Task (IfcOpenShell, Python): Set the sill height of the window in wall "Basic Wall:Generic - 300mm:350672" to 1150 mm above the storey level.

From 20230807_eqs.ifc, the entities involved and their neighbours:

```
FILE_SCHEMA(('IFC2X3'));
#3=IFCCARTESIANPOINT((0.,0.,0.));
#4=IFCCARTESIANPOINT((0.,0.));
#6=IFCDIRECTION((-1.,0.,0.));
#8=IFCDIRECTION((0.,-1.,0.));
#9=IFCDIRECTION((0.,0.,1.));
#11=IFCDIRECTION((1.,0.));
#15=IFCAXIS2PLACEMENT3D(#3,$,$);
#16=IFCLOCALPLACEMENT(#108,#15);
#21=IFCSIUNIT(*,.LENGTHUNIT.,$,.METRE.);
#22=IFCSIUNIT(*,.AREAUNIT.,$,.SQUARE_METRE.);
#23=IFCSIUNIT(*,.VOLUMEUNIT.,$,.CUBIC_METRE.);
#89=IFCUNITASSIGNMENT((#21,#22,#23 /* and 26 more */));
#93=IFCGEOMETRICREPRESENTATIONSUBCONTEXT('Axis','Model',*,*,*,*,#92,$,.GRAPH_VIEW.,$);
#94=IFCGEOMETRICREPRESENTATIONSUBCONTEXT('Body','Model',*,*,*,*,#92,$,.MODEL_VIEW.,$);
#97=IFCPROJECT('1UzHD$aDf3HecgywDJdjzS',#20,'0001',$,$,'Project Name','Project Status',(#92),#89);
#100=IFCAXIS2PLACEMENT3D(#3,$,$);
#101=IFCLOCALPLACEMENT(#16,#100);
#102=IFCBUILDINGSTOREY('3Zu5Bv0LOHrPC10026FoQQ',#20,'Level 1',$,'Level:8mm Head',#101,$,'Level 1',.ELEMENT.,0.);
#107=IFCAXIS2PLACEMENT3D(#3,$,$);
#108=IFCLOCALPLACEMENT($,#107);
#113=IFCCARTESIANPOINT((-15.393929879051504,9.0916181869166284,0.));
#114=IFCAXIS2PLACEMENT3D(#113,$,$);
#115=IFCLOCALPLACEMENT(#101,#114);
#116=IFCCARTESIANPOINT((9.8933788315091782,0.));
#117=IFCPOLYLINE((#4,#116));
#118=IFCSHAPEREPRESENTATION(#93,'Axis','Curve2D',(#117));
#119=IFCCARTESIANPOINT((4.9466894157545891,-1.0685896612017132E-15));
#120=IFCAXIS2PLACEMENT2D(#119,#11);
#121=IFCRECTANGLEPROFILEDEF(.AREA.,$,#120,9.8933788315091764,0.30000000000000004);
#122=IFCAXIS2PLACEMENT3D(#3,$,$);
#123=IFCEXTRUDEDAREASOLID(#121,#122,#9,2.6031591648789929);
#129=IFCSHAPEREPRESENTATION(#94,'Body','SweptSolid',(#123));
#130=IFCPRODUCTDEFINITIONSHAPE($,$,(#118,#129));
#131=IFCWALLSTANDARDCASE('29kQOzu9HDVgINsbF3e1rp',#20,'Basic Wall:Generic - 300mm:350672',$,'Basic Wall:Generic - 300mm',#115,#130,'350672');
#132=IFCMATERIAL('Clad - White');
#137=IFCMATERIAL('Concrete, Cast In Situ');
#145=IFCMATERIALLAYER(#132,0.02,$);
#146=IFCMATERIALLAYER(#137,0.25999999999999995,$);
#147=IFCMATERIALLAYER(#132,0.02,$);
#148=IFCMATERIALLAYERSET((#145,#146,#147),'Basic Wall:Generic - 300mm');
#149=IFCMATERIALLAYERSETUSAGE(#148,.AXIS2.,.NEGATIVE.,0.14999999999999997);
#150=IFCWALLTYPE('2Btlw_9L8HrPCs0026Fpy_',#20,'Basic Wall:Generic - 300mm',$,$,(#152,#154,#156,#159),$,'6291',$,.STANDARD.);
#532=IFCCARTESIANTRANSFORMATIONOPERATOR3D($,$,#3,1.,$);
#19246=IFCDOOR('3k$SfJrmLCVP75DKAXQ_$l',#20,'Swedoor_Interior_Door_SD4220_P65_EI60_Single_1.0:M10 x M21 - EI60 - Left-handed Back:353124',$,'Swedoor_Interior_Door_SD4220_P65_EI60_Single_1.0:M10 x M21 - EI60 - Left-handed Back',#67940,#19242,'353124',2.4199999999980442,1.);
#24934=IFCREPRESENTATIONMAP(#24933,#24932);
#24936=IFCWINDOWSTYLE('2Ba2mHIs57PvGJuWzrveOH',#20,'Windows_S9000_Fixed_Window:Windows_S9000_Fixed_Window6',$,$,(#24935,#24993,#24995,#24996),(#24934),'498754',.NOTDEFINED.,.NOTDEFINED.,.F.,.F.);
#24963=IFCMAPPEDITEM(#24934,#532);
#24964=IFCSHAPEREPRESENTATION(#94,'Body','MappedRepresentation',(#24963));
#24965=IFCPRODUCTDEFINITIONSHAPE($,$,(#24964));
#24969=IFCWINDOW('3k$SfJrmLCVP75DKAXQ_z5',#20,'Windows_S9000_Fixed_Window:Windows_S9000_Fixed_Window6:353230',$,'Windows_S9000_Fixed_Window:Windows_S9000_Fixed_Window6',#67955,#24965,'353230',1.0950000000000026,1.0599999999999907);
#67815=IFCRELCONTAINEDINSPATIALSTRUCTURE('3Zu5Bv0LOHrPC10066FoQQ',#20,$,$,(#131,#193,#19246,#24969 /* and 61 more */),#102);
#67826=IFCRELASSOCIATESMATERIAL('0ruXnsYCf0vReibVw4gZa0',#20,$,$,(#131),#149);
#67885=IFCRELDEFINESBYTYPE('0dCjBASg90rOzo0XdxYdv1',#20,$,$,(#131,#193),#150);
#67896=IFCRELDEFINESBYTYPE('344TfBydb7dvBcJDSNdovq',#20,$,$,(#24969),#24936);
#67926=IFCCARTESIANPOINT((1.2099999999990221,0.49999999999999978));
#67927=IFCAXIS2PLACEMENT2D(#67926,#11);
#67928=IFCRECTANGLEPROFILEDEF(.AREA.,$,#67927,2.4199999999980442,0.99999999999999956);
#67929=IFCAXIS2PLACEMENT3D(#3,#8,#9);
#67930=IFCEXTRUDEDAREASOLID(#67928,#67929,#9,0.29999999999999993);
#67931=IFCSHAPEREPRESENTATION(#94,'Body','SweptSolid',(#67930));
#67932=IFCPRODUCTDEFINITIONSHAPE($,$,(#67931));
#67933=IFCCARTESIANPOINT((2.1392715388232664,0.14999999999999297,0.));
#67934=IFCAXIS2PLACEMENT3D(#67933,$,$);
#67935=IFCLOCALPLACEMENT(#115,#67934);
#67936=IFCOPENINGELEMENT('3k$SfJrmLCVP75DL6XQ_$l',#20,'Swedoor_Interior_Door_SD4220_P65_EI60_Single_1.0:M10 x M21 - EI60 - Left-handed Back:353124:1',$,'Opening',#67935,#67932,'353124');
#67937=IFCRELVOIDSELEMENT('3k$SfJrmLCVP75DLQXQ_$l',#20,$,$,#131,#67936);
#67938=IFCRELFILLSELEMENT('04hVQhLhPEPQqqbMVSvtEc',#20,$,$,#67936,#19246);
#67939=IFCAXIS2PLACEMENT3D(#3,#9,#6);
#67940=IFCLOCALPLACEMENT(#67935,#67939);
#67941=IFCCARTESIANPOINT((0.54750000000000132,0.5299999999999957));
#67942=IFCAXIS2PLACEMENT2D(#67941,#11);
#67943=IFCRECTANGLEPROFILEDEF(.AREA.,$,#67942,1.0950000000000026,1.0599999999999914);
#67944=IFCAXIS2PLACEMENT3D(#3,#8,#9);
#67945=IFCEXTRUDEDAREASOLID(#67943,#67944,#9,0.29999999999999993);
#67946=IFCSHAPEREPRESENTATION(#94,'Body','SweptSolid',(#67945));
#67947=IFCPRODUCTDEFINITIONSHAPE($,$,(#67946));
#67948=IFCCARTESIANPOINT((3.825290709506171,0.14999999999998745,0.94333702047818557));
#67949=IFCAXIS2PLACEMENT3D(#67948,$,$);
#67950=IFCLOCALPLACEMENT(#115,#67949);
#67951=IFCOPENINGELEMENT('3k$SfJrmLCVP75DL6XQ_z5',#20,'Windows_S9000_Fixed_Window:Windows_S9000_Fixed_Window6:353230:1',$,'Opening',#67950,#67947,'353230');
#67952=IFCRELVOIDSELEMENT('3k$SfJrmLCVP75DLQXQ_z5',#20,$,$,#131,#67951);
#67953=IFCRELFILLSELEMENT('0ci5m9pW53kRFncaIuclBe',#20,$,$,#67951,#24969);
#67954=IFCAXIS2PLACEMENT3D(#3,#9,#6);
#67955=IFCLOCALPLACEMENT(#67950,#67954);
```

```python
import numpy as np
import ifcopenshell
import ifcopenshell.api.geometry
import ifcopenshell.geom
import ifcopenshell.util.element
import ifcopenshell.util.placement
import ifcopenshell.util.shape
import ifcopenshell.util.unit

model = ifcopenshell.open("20230807_eqs.ifc")
unit_scale = ifcopenshell.util.unit.calculate_unit_scale(model)

window = model.by_guid("3k$SfJrmLCVP75DKAXQ_z5")
opening = window.FillsVoids[0].RelatingOpeningElement
storey = ifcopenshell.util.element.get_container(window, ifc_class="IfcBuildingStorey")
level = ifcopenshell.util.placement.get_local_placement(storey.ObjectPlacement)[2, 3]

# The opening's origin need not be at the sill, so measure its lowest point.
shape = ifcopenshell.geom.create_shape(ifcopenshell.geom.settings(), opening)
bottom = ifcopenshell.util.shape.get_shape_bottom_elevation(shape, shape.geometry) / unit_scale
dz = level + 1.15 / unit_scale - bottom

shift = np.array([0.0, 0.0, dz])
# The window is placed relative to its opening, so it follows when the opening moves.
matrix = ifcopenshell.util.placement.get_local_placement(opening.ObjectPlacement)
matrix[:3, 3] += shift
ifcopenshell.api.geometry.edit_object_placement(
    model, product=opening, matrix=matrix, is_si=False, should_transform_children=True
)

print(f"moved by {dz * unit_scale:+.3f} m")

model.write("20230807_eqs_updated.ifc")
```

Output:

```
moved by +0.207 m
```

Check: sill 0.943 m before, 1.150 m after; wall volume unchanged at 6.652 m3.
